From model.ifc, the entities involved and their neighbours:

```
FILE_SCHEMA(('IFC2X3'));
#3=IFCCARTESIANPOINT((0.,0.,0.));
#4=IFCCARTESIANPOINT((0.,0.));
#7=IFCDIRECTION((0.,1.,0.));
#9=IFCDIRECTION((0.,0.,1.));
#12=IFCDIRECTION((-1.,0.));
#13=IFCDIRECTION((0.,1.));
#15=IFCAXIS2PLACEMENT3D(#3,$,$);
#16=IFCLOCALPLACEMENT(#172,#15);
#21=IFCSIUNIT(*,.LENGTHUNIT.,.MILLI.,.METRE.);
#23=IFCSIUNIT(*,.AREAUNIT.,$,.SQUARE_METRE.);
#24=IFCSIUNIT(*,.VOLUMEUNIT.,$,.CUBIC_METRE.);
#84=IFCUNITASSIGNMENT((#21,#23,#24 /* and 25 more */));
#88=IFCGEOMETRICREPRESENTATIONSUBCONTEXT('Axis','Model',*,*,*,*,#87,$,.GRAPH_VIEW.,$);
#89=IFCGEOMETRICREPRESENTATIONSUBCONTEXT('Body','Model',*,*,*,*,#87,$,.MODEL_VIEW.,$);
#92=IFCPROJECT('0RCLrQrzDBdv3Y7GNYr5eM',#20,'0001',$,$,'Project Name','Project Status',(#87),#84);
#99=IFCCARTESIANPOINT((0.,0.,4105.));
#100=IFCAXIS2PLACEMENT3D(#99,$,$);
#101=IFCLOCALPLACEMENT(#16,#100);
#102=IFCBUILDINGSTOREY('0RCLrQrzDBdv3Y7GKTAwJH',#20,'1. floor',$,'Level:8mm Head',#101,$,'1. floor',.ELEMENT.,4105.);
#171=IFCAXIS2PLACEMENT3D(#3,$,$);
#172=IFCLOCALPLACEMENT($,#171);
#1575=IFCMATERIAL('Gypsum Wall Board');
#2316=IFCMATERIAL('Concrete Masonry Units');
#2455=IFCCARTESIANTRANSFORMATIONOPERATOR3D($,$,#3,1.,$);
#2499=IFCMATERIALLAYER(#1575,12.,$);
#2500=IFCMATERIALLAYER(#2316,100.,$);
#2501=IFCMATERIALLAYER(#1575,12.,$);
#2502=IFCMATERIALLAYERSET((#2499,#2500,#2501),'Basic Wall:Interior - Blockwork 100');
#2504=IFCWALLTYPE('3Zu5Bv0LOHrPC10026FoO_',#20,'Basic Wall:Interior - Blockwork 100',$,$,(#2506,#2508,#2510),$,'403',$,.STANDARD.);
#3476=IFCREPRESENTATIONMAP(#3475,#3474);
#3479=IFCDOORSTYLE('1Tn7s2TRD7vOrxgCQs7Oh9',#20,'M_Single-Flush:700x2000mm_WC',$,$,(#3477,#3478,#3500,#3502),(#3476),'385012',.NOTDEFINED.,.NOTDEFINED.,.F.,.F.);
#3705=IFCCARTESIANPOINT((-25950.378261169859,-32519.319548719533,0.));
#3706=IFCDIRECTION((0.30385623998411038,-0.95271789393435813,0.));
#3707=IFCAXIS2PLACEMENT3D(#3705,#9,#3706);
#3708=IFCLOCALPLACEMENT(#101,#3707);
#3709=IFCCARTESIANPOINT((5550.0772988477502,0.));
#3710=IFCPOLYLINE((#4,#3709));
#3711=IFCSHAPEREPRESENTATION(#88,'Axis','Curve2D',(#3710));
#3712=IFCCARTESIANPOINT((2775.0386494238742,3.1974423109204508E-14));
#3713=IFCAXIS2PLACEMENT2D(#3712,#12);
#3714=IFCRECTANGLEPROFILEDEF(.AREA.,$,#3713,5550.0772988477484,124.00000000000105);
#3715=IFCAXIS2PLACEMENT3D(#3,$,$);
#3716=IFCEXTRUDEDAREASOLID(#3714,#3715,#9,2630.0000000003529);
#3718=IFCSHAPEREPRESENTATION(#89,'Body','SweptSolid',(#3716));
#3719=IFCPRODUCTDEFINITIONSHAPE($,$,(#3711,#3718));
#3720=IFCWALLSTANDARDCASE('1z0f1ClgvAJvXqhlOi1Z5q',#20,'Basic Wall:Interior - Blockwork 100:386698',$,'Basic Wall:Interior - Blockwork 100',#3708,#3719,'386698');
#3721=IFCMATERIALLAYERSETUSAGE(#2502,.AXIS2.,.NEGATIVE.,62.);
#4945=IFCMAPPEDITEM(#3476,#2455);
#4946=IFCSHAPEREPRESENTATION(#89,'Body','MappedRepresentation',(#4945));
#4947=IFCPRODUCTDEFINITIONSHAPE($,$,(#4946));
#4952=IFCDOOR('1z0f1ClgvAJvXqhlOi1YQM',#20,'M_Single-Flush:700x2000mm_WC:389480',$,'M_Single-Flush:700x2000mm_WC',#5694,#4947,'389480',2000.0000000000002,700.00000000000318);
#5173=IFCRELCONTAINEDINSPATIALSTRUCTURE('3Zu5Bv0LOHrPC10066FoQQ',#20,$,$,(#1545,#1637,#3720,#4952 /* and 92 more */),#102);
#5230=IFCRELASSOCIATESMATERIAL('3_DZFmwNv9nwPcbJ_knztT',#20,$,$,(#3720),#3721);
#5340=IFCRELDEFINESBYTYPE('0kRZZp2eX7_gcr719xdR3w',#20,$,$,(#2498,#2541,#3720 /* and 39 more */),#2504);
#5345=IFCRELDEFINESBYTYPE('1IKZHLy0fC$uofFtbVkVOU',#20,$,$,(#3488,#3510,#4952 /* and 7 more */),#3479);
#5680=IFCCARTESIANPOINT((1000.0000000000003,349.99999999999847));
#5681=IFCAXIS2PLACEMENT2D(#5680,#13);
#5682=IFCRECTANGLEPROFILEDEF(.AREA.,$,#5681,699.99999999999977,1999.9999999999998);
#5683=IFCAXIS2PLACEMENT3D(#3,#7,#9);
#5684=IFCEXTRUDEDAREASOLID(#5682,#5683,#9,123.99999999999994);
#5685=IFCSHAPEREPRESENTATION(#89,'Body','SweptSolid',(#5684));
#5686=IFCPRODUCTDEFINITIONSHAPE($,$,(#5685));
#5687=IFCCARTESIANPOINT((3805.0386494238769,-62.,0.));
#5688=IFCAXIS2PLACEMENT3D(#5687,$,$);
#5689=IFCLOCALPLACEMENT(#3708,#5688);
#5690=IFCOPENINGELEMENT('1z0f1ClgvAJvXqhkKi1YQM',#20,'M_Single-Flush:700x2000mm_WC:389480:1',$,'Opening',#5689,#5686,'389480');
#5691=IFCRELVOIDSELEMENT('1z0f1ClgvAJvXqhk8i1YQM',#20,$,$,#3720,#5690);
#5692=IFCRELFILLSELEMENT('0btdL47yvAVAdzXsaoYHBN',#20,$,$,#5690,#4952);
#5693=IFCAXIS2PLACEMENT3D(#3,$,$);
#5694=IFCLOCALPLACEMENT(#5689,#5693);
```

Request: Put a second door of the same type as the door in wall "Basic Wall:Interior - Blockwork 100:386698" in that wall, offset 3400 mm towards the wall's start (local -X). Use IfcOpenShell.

```python
import ifcopenshell
import ifcopenshell.api.feature
import ifcopenshell.api.geometry
import ifcopenshell.api.root
import ifcopenshell.geom
import ifcopenshell.util.element
import ifcopenshell.util.placement
import ifcopenshell.util.shape
import ifcopenshell.util.unit

model = ifcopenshell.open("model.ifc")
unit_scale = ifcopenshell.util.unit.calculate_unit_scale(model)
settings = ifcopenshell.geom.settings()


def volume(element):
    """Net volume in cubic metres, openings subtracted."""
    shape = ifcopenshell.geom.create_shape(settings, element)
    return ifcopenshell.util.shape.get_volume(shape.geometry)


def reuse_history(source, copy):
    """copy_class also copies each property set's owner history, people and application; keep the originals."""
    for rel in copy.IsDefinedBy:
        if rel.is_a("IfcRelDefinesByProperties") and (history := rel.RelatingPropertyDefinition.OwnerHistory):
            rel.RelatingPropertyDefinition.OwnerHistory = source.OwnerHistory
            ifcopenshell.util.element.remove_deep2(model, history)


door = model.by_guid("1z0f1ClgvAJvXqhlOi1YQM")
opening = door.FillsVoids[0].RelatingOpeningElement
wall = opening.VoidsElements[0].RelatingBuildingElement
before = volume(wall)
shift = ifcopenshell.util.placement.get_local_placement(wall.ObjectPlacement)[:3, 0] * -3.4 / unit_scale

# copy_class copies the void relationship, type, container and properties, but no geometry.
new_opening = ifcopenshell.api.root.copy_class(model, product=opening)
new_opening.Representation = ifcopenshell.util.element.copy_deep(
    model, opening.Representation, exclude=["IfcGeometricRepresentationContext", "IfcRepresentationMap"]
)
new_opening.Name = "M_Single-Flush:700x2000mm_WC"
new_opening.Tag = None
new_door = ifcopenshell.api.root.copy_class(model, product=door)
new_door.Representation = ifcopenshell.util.element.copy_deep(
    model, door.Representation, exclude=["IfcGeometricRepresentationContext", "IfcRepresentationMap"]
)
new_door.Name = "M_Single-Flush:700x2000mm_WC"
new_door.Tag = None
reuse_history(door, new_door)
fills = ifcopenshell.api.feature.add_filling(model, opening=new_opening, element=new_door)
fills.OwnerHistory = new_door.OwnerHistory  # required in IFC2X3

for old, new in ((opening, new_opening), (door, new_door)):
    matrix = ifcopenshell.util.placement.get_local_placement(old.ObjectPlacement)
    matrix[:3, 3] += shift
    ifcopenshell.api.geometry.edit_object_placement(model, product=new, matrix=matrix, is_si=False)

after = volume(wall)

print(f"wall volume {before:.3f} -> {after:.3f} m3")

model.write("model-out.ifc")
```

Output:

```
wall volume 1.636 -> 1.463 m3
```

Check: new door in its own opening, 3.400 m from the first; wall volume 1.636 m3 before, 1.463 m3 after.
